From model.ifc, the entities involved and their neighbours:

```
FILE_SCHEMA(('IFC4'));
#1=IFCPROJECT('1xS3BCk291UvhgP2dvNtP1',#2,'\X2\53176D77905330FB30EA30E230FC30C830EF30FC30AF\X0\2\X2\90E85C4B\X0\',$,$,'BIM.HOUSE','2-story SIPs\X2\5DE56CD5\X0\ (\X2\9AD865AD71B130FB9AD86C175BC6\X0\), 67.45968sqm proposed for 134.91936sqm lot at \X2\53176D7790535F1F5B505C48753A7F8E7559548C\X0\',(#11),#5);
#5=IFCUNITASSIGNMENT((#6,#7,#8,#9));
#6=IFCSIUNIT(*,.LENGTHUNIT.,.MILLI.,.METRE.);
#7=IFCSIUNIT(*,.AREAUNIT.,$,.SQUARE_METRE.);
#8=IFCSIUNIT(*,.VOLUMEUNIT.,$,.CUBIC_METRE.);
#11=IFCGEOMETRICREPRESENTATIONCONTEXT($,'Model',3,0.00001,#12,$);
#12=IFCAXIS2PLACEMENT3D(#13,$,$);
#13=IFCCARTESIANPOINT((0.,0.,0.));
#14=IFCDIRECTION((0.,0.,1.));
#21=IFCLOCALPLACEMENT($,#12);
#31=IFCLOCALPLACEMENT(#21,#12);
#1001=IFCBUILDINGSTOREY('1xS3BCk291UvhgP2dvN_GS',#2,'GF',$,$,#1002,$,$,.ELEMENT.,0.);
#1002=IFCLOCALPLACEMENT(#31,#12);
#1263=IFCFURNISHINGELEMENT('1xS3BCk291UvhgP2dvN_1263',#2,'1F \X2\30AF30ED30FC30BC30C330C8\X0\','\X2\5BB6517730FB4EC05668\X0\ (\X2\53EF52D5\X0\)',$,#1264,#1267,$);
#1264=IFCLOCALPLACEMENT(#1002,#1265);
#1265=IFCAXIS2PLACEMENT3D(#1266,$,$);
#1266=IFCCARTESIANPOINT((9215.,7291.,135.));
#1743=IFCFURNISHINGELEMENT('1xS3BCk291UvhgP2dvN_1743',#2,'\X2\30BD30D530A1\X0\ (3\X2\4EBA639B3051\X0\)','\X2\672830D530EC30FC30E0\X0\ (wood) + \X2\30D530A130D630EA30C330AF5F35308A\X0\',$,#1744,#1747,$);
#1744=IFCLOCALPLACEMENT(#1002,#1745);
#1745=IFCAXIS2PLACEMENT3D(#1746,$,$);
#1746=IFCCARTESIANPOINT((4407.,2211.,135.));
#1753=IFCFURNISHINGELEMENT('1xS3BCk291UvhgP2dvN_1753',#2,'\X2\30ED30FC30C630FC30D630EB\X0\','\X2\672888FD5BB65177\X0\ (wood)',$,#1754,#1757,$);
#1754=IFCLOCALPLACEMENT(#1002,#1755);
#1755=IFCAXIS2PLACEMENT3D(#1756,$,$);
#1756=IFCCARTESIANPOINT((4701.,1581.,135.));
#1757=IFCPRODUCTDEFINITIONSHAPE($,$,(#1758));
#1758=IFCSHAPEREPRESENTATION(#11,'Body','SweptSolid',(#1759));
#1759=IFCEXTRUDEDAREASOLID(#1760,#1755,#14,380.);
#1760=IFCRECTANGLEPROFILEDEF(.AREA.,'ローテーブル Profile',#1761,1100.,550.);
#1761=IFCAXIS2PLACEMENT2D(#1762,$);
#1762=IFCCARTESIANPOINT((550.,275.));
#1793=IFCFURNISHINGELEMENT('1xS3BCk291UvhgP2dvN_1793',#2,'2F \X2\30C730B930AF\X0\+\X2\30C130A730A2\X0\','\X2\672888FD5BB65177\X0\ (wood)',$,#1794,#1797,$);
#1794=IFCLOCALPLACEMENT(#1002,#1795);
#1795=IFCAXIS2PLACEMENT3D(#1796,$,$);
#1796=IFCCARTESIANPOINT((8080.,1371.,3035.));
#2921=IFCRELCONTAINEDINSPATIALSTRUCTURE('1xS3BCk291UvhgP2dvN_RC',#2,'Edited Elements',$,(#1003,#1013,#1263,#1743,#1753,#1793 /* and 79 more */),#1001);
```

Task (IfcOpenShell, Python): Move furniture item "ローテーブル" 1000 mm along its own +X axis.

```python
import ifcopenshell
import ifcopenshell.api.geometry
import ifcopenshell.util.placement
import ifcopenshell.util.unit

model = ifcopenshell.open("model.ifc")
unit_scale = ifcopenshell.util.unit.calculate_unit_scale(model)

item = model.by_guid("1xS3BCk291UvhgP2dvN_1753")
matrix = ifcopenshell.util.placement.get_local_placement(item.ObjectPlacement)
matrix[:3, 3] += matrix[:3, 0] * 1 / unit_scale
ifcopenshell.api.geometry.edit_object_placement(model, product=item, matrix=matrix, is_si=False)

print(ifcopenshell.util.placement.get_local_placement(item.ObjectPlacement).round(3) + 0.0)

model.write("model_rev.ifc")
```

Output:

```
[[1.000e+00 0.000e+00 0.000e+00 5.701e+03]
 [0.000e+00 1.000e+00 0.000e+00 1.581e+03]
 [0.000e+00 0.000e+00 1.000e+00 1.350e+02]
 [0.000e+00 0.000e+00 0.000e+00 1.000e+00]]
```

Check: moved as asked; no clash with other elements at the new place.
